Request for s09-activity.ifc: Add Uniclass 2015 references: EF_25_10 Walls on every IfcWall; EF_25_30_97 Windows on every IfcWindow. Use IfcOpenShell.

First a look at what the model holds.

```python
import ifcopenshell

model = ifcopenshell.open("s09-activity.ifc")
print(model.schema)
print("classifications:", [c.Name for c in model.by_type("IfcClassification")])
for ifc_class in ("IfcDoor", "IfcRoof", "IfcStair", "IfcWall", "IfcWindow"):
    print(ifc_class, len(model.by_type(ifc_class)))
```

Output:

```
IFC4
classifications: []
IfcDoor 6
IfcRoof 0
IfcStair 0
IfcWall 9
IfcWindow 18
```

```python
import ifcopenshell
import ifcopenshell.api.classification

model = ifcopenshell.open("s09-activity.ifc")

system = ifcopenshell.api.classification.add_classification(model, classification="Uniclass 2015")

codes = {
    "IfcWall": ("EF_25_10", "Walls"),
    "IfcWindow": ("EF_25_30_97", "Windows"),
}
for ifc_class, (code, name) in codes.items():
    products = model.by_type(ifc_class)
    ifcopenshell.api.classification.add_reference(
        model, products=products, classification=system, identification=code, name=name
    )
    print(code, len(products))

model.write("s09-activity-out.ifc")
```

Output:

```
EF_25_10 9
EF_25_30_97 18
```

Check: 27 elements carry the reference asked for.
